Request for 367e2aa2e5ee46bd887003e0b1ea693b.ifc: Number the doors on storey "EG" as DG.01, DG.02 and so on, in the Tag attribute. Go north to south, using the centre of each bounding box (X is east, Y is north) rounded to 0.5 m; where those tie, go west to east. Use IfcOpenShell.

First a look at what the model holds.

```python
import ifcopenshell
import ifcopenshell.util.element
import ifcopenshell.util.placement

model = ifcopenshell.open("367e2aa2e5ee46bd887003e0b1ea693b.ifc")
print(model.schema)
storey = next(s for s in model.by_type("IfcBuildingStorey") if s.Name == "EG")
doors = [e for e in ifcopenshell.util.element.get_decomposition(storey) if e.is_a("IfcDoor")]
for e in sorted(doors, key=lambda e: e.id()):
    origin = ifcopenshell.util.placement.get_local_placement(e.ObjectPlacement)[:3, 3]
    print(e.id(), e.Tag, e.Name, origin.round(2) + 0.0, sep=" | ")
```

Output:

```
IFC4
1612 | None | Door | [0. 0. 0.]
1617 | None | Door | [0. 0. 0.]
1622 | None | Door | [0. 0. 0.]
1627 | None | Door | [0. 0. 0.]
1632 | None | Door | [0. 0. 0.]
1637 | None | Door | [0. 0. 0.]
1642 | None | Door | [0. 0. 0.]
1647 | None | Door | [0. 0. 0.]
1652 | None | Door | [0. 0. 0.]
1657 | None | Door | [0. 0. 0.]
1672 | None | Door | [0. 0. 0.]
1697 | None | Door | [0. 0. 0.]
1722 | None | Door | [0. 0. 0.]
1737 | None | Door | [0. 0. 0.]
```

```python
import ifcopenshell
import ifcopenshell.geom
import ifcopenshell.util.element
import ifcopenshell.util.shape

model = ifcopenshell.open("367e2aa2e5ee46bd887003e0b1ea693b.ifc")
settings = ifcopenshell.geom.settings()
settings.set("use-world-coords", True)


def centre(element):
    shape = ifcopenshell.geom.create_shape(settings, element)
    return ifcopenshell.util.shape.get_bbox_centroid(shape.geometry)


storey = next(s for s in model.by_type("IfcBuildingStorey") if s.Name == "EG")
doors = [e for e in ifcopenshell.util.element.get_decomposition(storey) if e.is_a("IfcDoor")]

# Insertion points can sit at a corner or the storey origin, so sort by the geometry (in metres).
centres = {e: centre(e) for e in doors}
doors.sort(key=lambda e: (-round(centres[e][1] / 0.5), centres[e][0]))

for i, e in enumerate(doors, start=1):
    number = f"DG.{i:02d}"
    e.Tag = number
    print(e.id(), number)

model.write("367e2aa2e5ee46bd887003e0b1ea693b-out.ifc")
```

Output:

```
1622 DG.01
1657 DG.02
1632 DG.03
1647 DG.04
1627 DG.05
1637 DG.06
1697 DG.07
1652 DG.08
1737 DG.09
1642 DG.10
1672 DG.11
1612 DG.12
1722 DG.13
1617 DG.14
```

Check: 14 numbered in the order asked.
